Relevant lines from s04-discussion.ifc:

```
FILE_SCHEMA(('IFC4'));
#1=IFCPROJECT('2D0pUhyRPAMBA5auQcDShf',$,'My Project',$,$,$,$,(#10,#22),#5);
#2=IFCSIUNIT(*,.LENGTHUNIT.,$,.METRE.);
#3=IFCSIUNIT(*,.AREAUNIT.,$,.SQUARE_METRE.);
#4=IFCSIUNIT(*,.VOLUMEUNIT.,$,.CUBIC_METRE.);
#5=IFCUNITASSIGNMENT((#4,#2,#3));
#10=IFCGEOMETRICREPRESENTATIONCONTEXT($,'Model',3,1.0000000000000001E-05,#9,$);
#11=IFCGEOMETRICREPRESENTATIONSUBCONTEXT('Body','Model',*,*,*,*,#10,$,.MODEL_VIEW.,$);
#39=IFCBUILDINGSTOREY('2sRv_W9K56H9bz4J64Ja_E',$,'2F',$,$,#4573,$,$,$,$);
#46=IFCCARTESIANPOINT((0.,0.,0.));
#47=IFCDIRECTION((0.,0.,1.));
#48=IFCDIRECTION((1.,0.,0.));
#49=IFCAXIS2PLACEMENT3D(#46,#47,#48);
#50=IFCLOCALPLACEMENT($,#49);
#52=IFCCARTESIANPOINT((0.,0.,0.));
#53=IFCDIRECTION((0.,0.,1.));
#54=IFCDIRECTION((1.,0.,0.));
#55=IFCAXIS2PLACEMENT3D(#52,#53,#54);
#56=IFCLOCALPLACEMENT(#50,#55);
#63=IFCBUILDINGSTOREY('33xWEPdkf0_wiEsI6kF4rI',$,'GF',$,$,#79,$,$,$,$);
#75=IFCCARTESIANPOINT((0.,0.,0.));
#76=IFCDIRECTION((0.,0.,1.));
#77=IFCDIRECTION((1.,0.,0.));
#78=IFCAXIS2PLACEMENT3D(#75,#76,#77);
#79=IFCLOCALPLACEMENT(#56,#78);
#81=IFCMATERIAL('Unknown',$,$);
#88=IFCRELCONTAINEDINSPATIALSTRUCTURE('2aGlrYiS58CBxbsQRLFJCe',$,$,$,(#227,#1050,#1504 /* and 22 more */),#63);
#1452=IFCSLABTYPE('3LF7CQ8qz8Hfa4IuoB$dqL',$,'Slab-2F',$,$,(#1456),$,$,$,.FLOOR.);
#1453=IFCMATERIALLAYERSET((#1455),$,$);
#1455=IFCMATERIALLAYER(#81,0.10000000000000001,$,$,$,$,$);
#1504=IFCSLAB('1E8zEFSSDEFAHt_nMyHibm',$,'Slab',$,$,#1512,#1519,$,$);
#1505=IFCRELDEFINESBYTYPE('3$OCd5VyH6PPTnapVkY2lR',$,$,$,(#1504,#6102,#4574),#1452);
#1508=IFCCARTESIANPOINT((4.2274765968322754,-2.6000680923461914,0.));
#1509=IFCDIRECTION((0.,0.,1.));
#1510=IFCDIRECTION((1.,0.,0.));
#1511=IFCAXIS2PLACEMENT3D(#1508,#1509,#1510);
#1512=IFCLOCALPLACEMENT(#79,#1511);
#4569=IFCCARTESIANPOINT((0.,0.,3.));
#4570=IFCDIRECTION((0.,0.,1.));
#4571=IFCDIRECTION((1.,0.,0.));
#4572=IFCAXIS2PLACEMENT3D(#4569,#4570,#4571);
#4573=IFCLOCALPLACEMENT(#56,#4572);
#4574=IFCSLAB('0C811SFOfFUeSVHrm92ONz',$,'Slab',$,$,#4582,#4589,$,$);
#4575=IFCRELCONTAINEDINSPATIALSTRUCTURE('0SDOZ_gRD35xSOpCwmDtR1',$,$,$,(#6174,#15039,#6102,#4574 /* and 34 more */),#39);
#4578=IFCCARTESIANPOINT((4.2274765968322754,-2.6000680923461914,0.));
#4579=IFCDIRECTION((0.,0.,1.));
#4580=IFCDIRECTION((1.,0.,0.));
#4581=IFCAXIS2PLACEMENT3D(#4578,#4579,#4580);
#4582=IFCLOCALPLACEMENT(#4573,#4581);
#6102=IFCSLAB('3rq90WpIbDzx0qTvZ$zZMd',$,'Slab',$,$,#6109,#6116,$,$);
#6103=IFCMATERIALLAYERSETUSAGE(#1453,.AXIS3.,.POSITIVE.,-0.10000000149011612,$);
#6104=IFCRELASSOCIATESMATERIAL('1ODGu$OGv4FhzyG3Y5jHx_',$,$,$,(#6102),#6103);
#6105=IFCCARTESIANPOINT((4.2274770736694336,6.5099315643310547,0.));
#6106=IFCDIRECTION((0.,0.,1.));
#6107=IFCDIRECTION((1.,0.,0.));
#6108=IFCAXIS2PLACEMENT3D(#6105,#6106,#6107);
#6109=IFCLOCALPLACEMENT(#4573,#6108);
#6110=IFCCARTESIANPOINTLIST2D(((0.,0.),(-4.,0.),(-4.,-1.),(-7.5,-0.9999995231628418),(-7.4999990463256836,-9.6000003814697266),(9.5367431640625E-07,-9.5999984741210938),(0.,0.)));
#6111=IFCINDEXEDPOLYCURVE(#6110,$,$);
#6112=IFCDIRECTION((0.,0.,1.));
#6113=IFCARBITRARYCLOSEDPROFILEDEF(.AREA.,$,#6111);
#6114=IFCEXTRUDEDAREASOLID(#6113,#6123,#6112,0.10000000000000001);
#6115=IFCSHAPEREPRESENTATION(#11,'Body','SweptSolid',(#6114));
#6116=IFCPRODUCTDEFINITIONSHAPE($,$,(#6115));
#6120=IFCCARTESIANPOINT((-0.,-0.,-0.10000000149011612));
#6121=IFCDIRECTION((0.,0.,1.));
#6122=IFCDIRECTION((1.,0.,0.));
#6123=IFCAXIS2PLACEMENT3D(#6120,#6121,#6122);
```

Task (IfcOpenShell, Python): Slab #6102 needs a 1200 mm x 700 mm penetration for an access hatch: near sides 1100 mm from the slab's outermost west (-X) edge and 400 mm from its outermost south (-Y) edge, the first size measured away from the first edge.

```python
import numpy as np
import ifcopenshell
import ifcopenshell.api.feature
import ifcopenshell.api.geometry
import ifcopenshell.api.root
import ifcopenshell.geom
import ifcopenshell.util.placement
import ifcopenshell.util.representation
import ifcopenshell.util.shape
import ifcopenshell.util.unit

model = ifcopenshell.open("s04-discussion.ifc")
unit_scale = ifcopenshell.util.unit.calculate_unit_scale(model)
settings = ifcopenshell.geom.settings()


def volume(element):
    """Net volume in cubic metres, openings subtracted."""
    shape = ifcopenshell.geom.create_shape(settings, element)
    return ifcopenshell.util.shape.get_volume(shape.geometry)


slab = model.by_guid("3rq90WpIbDzx0qTvZ$zZMd")
before = volume(slab)

# Extent in the slab's own axes, in metres. The edges named are its -X and -Y sides.
slab_shape = ifcopenshell.geom.create_shape(settings, slab)
vertices = ifcopenshell.util.shape.get_vertices(slab_shape.geometry)
x_min, y_min, bottom = vertices.min(axis=0)
top = vertices[:, 2].max()

opening = ifcopenshell.api.root.create_entity(model, ifc_class="IfcOpeningElement", name="Access hatch opening", predefined_type="OPENING")
context = ifcopenshell.util.representation.get_context(model, "Model", "Body", "MODEL_VIEW")
width, depth = 1.2, 0.7
outline = [(0.0, 0.0), (width, 0.0), (width, depth), (0.0, depth), (0.0, 0.0)]
# Overshoot both faces by 50 mm so the cut is clean.
shape = ifcopenshell.api.geometry.add_slab_representation(
    model, context=context, depth=top - bottom + 0.1, polyline=outline
)
ifcopenshell.api.geometry.assign_representation(model, product=opening, representation=shape)

matrix = ifcopenshell.util.placement.get_local_placement(slab.ObjectPlacement)
matrix[:, 3] = matrix @ np.append(np.array([x_min + 1.1, y_min + 0.4, bottom - 0.05]) / unit_scale, 1.0)
ifcopenshell.api.geometry.edit_object_placement(model, product=opening, matrix=matrix, is_si=False)
ifcopenshell.api.feature.add_feature(model, feature=opening, element=slab)

after = volume(slab)

print(f"slab volume {before:.3f} -> {after:.3f} m3")

model.write("s04-discussion_updated.ifc")
```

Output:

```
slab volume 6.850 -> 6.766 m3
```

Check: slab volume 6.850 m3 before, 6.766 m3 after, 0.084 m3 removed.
